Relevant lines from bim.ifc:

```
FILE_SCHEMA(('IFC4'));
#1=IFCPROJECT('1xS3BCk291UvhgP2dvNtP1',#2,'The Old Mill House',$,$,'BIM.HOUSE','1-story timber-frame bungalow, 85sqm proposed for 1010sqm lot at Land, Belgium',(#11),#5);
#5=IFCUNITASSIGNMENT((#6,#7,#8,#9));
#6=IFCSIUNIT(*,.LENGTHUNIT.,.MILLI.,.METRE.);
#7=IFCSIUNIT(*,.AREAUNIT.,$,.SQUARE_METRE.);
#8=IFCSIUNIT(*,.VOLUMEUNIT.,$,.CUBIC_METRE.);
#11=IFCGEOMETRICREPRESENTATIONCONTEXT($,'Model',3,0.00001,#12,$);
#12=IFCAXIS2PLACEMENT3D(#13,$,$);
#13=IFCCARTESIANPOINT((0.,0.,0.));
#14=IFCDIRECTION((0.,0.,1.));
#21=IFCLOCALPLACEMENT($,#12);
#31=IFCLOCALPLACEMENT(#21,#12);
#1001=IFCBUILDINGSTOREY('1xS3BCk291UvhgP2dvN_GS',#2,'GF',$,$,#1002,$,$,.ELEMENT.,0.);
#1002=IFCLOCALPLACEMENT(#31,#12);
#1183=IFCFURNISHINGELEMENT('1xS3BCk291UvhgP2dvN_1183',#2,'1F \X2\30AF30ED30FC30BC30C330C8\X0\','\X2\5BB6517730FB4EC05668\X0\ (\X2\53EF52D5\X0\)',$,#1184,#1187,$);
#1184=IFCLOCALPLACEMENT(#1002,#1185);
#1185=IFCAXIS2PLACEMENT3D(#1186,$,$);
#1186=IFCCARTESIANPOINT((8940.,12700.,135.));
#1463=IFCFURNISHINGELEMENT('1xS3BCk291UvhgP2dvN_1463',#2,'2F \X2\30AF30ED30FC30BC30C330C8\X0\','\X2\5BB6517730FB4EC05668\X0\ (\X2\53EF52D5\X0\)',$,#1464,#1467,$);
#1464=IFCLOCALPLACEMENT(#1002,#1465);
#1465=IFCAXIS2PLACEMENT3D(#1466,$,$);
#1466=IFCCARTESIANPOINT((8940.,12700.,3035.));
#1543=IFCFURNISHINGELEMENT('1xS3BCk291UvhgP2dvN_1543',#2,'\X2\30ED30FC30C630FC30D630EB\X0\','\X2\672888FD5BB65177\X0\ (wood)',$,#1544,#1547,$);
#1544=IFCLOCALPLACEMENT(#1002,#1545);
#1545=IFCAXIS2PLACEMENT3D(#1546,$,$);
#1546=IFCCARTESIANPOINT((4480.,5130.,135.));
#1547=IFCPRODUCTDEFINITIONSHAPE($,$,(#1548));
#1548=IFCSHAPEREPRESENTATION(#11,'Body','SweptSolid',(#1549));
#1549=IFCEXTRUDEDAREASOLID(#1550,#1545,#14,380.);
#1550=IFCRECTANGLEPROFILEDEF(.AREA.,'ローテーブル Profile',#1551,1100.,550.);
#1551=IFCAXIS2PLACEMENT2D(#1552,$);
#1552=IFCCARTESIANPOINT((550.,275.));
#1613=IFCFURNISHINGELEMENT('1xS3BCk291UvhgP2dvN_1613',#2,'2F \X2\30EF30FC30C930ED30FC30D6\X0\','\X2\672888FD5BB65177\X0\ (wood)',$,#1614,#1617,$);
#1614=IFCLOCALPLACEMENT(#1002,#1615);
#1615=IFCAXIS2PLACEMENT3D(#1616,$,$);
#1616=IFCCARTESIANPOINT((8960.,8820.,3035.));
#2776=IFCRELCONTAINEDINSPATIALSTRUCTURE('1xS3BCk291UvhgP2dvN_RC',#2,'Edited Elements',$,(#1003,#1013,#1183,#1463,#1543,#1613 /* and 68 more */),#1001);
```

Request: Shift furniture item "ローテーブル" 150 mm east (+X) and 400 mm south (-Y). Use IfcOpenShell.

```python
import ifcopenshell
import ifcopenshell.api.geometry
import ifcopenshell.util.placement
import ifcopenshell.util.unit

model = ifcopenshell.open("bim.ifc")
unit_scale = ifcopenshell.util.unit.calculate_unit_scale(model)

item = model.by_guid("1xS3BCk291UvhgP2dvN_1543")
matrix = ifcopenshell.util.placement.get_local_placement(item.ObjectPlacement)
matrix[0, 3] += 0.15 / unit_scale
matrix[1, 3] -= 0.4 / unit_scale
ifcopenshell.api.geometry.edit_object_placement(model, product=item, matrix=matrix, is_si=False)

print(ifcopenshell.util.placement.get_local_placement(item.ObjectPlacement).round(3) + 0.0)

model.write("bim_updated.ifc")
```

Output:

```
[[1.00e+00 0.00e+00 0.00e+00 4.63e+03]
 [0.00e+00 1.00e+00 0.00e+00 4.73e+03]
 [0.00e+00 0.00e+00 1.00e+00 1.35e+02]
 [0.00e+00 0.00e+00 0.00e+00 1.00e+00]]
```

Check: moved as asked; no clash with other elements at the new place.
